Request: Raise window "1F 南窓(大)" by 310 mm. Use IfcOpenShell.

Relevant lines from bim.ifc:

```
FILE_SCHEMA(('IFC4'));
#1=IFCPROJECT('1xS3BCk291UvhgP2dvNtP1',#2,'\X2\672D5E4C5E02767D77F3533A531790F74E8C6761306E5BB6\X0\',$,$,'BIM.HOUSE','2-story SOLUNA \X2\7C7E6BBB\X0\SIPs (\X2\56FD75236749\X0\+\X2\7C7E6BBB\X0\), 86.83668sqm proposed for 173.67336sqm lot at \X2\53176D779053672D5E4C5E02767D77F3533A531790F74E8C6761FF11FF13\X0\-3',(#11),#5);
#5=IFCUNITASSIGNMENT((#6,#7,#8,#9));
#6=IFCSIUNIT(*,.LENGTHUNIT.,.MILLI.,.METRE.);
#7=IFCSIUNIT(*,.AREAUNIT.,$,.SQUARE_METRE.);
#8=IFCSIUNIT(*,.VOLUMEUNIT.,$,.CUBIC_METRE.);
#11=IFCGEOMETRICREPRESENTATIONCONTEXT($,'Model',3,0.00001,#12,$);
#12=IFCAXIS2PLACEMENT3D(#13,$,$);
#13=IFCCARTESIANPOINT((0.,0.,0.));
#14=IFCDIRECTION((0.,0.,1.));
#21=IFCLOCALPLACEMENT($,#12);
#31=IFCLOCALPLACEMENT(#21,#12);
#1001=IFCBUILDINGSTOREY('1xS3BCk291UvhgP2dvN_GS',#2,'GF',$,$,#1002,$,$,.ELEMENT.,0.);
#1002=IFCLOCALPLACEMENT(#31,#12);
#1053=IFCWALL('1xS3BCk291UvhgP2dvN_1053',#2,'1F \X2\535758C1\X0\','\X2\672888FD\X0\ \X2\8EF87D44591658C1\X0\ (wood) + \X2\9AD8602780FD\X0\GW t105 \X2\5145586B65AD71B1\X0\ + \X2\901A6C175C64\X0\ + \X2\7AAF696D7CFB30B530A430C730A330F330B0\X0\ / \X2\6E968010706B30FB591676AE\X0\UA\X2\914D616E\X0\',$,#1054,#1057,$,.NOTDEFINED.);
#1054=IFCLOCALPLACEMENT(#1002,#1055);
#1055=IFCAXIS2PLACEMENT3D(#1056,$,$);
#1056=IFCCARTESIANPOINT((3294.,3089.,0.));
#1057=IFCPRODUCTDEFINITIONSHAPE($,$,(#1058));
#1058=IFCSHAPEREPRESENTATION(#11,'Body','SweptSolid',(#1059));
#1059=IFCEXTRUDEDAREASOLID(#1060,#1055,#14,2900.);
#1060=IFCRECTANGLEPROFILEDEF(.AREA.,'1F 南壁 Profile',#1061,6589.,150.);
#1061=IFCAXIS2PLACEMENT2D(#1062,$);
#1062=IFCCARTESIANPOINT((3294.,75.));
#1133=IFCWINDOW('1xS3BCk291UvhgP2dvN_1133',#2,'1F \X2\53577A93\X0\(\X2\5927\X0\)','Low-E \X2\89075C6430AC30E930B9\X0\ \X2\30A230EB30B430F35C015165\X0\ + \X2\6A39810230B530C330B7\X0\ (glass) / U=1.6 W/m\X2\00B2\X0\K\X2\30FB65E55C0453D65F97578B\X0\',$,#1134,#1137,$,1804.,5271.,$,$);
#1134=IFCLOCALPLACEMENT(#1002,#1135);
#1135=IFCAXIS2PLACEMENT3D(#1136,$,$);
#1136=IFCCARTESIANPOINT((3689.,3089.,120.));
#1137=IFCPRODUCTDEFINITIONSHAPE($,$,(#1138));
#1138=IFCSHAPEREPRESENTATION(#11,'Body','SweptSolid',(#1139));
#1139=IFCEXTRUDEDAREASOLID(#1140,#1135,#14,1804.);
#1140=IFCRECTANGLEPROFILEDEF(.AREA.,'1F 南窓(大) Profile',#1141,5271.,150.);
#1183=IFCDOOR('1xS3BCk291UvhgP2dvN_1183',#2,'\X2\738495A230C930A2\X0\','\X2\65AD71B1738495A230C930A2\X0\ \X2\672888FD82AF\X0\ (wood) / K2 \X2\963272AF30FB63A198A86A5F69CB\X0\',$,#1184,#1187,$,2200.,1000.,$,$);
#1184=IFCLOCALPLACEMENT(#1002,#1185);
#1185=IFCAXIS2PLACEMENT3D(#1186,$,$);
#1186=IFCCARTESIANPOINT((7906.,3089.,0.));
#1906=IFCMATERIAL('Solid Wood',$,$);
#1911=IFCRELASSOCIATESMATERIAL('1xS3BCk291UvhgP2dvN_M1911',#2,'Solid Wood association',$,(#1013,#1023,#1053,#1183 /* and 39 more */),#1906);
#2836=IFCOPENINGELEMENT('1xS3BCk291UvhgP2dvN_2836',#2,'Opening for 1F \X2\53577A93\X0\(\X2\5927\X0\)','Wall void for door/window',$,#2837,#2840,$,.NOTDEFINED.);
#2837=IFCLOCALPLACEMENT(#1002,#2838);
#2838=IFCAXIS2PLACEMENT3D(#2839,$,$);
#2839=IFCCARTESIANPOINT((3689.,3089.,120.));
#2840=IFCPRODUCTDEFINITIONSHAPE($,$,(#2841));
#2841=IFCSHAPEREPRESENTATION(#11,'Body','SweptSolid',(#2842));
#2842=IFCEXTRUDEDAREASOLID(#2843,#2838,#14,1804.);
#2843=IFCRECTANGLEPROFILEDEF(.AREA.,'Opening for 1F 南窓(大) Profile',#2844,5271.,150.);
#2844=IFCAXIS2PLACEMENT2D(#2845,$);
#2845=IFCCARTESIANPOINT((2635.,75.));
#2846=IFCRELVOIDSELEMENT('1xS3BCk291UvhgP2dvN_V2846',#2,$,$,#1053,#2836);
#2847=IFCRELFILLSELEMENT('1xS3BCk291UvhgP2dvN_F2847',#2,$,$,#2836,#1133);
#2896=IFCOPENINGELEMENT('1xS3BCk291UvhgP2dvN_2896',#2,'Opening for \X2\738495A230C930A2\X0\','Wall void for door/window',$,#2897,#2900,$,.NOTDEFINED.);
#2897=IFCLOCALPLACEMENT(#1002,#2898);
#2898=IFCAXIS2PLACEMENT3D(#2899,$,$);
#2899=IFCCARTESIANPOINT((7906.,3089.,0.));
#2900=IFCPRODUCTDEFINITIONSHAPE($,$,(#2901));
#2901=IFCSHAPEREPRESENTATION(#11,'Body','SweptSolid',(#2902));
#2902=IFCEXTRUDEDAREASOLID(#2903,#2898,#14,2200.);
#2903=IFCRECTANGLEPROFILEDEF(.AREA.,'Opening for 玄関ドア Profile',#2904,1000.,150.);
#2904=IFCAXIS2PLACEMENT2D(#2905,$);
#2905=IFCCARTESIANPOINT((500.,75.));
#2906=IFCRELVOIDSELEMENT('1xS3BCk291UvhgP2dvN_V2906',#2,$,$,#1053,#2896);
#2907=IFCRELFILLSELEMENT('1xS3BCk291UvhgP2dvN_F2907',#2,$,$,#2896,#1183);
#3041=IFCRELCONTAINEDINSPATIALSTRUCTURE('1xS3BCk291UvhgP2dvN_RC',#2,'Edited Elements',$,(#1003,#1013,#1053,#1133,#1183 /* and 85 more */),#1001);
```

```python
import numpy as np
import ifcopenshell
import ifcopenshell.api.geometry
import ifcopenshell.util.placement
import ifcopenshell.util.unit

model = ifcopenshell.open("bim.ifc")
unit_scale = ifcopenshell.util.unit.calculate_unit_scale(model)

window = model.by_guid("1xS3BCk291UvhgP2dvN_1133")
opening = window.FillsVoids[0].RelatingOpeningElement
dz = 0.31 / unit_scale

shift = np.array([0.0, 0.0, dz])
# The window is not placed relative to its opening, so move both.
for product in (opening, window):
    matrix = ifcopenshell.util.placement.get_local_placement(product.ObjectPlacement)
    matrix[:3, 3] += shift
    ifcopenshell.api.geometry.edit_object_placement(model, product=product, matrix=matrix, is_si=False)

print(f"moved by {dz * unit_scale:+.3f} m")

model.write("bim_updated.ifc")
```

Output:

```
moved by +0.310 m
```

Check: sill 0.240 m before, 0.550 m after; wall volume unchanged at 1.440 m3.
